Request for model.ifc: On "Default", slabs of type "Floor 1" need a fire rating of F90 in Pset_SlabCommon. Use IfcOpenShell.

First a look at what the model holds.

```python
import ifcopenshell
import ifcopenshell.util.element

model = ifcopenshell.open("model.ifc")
print(model.schema)
storey = next(s for s in model.by_type("IfcBuildingStorey") if s.Name == "Default")
slabs = [e for e in ifcopenshell.util.element.get_decomposition(storey) if e.is_a("IfcSlab")]
seen = {}
for e in slabs:
    element_type = ifcopenshell.util.element.get_type(e)
    key = (element_type.Name if element_type != e and element_type else None, ifcopenshell.util.element.get_pset(e, "Pset_SlabCommon", "FireRating"))
    seen[key] = seen.get(key, 0) + 1
for (name, value), count in sorted(seen.items(), key=str):
    print(count, "x", name, "|", value)
```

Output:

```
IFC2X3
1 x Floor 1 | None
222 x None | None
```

```python
import ifcopenshell
import ifcopenshell.api.pset
import ifcopenshell.util.element

model = ifcopenshell.open("model.ifc")

storey = next(s for s in model.by_type("IfcBuildingStorey") if s.Name == "Default")
slabs = [e for e in ifcopenshell.util.element.get_decomposition(storey) if e.is_a("IfcSlab")]

count = 0
for e in slabs:
    element_type = ifcopenshell.util.element.get_type(e)
    if element_type in (None, e) or element_type.Name != "Floor 1":
        continue
    # add_pset returns the element's existing set when there is one.
    pset = ifcopenshell.api.pset.add_pset(model, product=e, name="Pset_SlabCommon")
    ifcopenshell.api.pset.edit_pset(model, pset=pset, properties={"FireRating": "F90"})
    count += 1

print(count, "slabs updated")

model.write("model_edited.ifc")
```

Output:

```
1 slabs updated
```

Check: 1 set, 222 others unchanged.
